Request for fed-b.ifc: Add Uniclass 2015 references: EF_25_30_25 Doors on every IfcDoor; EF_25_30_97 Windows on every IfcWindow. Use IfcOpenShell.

First a look at what the model holds.

```python
import ifcopenshell

model = ifcopenshell.open("fed-b.ifc")
print(model.schema)
print("classifications:", [c.Name for c in model.by_type("IfcClassification")])
for ifc_class in ("IfcDoor", "IfcRoof", "IfcStair", "IfcWall", "IfcWindow"):
    print(ifc_class, len(model.by_type(ifc_class)))
```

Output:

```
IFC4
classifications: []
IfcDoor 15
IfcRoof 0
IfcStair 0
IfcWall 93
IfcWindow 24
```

```python
import ifcopenshell
import ifcopenshell.api.classification

model = ifcopenshell.open("fed-b.ifc")

system = ifcopenshell.api.classification.add_classification(model, classification="Uniclass 2015")

codes = {
    "IfcDoor": ("EF_25_30_25", "Doors"),
    "IfcWindow": ("EF_25_30_97", "Windows"),
}
for ifc_class, (code, name) in codes.items():
    products = model.by_type(ifc_class)
    ifcopenshell.api.classification.add_reference(
        model, products=products, classification=system, identification=code, name=name
    )
    print(code, len(products))

model.write("fed-b_updated.ifc")
```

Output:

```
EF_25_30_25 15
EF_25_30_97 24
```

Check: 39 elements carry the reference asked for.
